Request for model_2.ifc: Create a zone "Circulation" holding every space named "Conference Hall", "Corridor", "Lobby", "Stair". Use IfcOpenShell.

First a look at what the model holds.

```python
import ifcopenshell

model = ifcopenshell.open("model_2.ifc")
print(model.schema)
seen = {}
for space in model.by_type("IfcSpace"):
    seen[space.LongName] = seen.get(space.LongName, 0) + 1
for name, count in sorted(seen.items(), key=str):
    print(count, "x", name)
print("zones:", [z.Name for z in model.by_type("IfcZone")][:20])
```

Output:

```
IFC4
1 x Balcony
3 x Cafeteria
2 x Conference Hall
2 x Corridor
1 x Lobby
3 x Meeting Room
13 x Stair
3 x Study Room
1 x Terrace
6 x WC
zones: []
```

```python
import ifcopenshell
import ifcopenshell.api.group
import ifcopenshell.api.root

model = ifcopenshell.open("model_2.ifc")

names = {"Conference Hall", "Corridor", "Lobby", "Stair"}
spaces = [s for s in model.by_type("IfcSpace") if s.LongName in names]

zone = ifcopenshell.api.root.create_entity(model, ifc_class="IfcZone", name="Circulation")
ifcopenshell.api.group.assign_group(model, products=spaces, group=zone)
print(len(spaces), "spaces in", zone.Name)

model.write("model_2_edited.ifc")
```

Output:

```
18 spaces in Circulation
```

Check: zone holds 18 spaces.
